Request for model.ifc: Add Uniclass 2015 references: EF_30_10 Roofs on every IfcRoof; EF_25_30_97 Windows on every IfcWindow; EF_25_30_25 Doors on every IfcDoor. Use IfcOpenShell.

First a look at what the model holds.

```python
import ifcopenshell

model = ifcopenshell.open("model.ifc")
print(model.schema)
print("classifications:", [c.Name for c in model.by_type("IfcClassification")])
for ifc_class in ("IfcDoor", "IfcRoof", "IfcStair", "IfcWall", "IfcWindow"):
    print(ifc_class, len(model.by_type(ifc_class)))
```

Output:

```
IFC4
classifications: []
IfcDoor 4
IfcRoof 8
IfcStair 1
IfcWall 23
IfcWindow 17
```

```python
import ifcopenshell
import ifcopenshell.api.classification

model = ifcopenshell.open("model.ifc")

system = ifcopenshell.api.classification.add_classification(model, classification="Uniclass 2015")

codes = {
    "IfcRoof": ("EF_30_10", "Roofs"),
    "IfcWindow": ("EF_25_30_97", "Windows"),
    "IfcDoor": ("EF_25_30_25", "Doors"),
}
for ifc_class, (code, name) in codes.items():
    products = model.by_type(ifc_class)
    ifcopenshell.api.classification.add_reference(
        model, products=products, classification=system, identification=code, name=name
    )
    print(code, len(products))

model.write("model-out.ifc")
```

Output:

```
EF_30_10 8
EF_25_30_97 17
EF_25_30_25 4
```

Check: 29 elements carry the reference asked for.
